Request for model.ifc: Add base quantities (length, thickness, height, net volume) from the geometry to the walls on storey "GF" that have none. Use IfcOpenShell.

First a look at what the model holds.

```python
import ifcopenshell
import ifcopenshell.util.element
import ifcopenshell.util.unit

model = ifcopenshell.open("model.ifc")
print(model.schema)
for unit_type in ("LENGTHUNIT", "AREAUNIT", "VOLUMEUNIT"):
    print(unit_type, ifcopenshell.util.unit.calculate_unit_scale(model, unit_type))
storey = next(s for s in model.by_type("IfcBuildingStorey") if s.Name == "GF")
walls = [e for e in ifcopenshell.util.element.get_decomposition(storey) if e.is_a("IfcWall")]
for e in sorted(walls, key=lambda e: e.id()):
    print(e.id(), e.is_a(), e.Name, list(ifcopenshell.util.element.get_psets(e, qtos_only=True)), sep=" | ")
```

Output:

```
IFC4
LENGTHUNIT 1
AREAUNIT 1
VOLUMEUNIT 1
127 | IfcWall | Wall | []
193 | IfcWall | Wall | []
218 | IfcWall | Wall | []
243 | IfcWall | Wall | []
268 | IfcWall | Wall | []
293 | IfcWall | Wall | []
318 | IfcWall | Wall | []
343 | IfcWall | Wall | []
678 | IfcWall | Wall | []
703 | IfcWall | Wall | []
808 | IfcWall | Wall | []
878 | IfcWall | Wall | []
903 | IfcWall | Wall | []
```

```python
import ifcopenshell
import ifcopenshell.api.pset
import ifcopenshell.geom
import ifcopenshell.util.element
import ifcopenshell.util.shape
import ifcopenshell.util.unit

model = ifcopenshell.open("model.ifc")
unit_scale = ifcopenshell.util.unit.calculate_unit_scale(model)
volume_scale = ifcopenshell.util.unit.calculate_unit_scale(model, "VOLUMEUNIT")
settings = ifcopenshell.geom.settings()

storey = next(s for s in model.by_type("IfcBuildingStorey") if s.Name == "GF")
walls = [e for e in ifcopenshell.util.element.get_decomposition(storey) if e.is_a("IfcWall")]

for e in sorted(walls, key=lambda e: e.id()):
    if ifcopenshell.util.element.get_psets(e, qtos_only=True, should_inherit=False):
        continue
    # Geometry comes back in metres, in the element's own axes.
    shape = ifcopenshell.geom.create_shape(settings, e)
    values = {
        "Length": ifcopenshell.util.shape.get_x(shape.geometry) / unit_scale,
        "Width": ifcopenshell.util.shape.get_y(shape.geometry) / unit_scale,
        "Height": ifcopenshell.util.shape.get_z(shape.geometry) / unit_scale,
        "NetVolume": ifcopenshell.util.shape.get_volume(shape.geometry) / volume_scale,
    }
    qto = ifcopenshell.api.pset.add_qto(model, product=e, name="Qto_WallBaseQuantities")
    ifcopenshell.api.pset.edit_qto(model, qto=qto, properties=values)
    print(e.id(), {k: round(v, 3) for k, v in values.items()})

model.write("model-out.ifc")
```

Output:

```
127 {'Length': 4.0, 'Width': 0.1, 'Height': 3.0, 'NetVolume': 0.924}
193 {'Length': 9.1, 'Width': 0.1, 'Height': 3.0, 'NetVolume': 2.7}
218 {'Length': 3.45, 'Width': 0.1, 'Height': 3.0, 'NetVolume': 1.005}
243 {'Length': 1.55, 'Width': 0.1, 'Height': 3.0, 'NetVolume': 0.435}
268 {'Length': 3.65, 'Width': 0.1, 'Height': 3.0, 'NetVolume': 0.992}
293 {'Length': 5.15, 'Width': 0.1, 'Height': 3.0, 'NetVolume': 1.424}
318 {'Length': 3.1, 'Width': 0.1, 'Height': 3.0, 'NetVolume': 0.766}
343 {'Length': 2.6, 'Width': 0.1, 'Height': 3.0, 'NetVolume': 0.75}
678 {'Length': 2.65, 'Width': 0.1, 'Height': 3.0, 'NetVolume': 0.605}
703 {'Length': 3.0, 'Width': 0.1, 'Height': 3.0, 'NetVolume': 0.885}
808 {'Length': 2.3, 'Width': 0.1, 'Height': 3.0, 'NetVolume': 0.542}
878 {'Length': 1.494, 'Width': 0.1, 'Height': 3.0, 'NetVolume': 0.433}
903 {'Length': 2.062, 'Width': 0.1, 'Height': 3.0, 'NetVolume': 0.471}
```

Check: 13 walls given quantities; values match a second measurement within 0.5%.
